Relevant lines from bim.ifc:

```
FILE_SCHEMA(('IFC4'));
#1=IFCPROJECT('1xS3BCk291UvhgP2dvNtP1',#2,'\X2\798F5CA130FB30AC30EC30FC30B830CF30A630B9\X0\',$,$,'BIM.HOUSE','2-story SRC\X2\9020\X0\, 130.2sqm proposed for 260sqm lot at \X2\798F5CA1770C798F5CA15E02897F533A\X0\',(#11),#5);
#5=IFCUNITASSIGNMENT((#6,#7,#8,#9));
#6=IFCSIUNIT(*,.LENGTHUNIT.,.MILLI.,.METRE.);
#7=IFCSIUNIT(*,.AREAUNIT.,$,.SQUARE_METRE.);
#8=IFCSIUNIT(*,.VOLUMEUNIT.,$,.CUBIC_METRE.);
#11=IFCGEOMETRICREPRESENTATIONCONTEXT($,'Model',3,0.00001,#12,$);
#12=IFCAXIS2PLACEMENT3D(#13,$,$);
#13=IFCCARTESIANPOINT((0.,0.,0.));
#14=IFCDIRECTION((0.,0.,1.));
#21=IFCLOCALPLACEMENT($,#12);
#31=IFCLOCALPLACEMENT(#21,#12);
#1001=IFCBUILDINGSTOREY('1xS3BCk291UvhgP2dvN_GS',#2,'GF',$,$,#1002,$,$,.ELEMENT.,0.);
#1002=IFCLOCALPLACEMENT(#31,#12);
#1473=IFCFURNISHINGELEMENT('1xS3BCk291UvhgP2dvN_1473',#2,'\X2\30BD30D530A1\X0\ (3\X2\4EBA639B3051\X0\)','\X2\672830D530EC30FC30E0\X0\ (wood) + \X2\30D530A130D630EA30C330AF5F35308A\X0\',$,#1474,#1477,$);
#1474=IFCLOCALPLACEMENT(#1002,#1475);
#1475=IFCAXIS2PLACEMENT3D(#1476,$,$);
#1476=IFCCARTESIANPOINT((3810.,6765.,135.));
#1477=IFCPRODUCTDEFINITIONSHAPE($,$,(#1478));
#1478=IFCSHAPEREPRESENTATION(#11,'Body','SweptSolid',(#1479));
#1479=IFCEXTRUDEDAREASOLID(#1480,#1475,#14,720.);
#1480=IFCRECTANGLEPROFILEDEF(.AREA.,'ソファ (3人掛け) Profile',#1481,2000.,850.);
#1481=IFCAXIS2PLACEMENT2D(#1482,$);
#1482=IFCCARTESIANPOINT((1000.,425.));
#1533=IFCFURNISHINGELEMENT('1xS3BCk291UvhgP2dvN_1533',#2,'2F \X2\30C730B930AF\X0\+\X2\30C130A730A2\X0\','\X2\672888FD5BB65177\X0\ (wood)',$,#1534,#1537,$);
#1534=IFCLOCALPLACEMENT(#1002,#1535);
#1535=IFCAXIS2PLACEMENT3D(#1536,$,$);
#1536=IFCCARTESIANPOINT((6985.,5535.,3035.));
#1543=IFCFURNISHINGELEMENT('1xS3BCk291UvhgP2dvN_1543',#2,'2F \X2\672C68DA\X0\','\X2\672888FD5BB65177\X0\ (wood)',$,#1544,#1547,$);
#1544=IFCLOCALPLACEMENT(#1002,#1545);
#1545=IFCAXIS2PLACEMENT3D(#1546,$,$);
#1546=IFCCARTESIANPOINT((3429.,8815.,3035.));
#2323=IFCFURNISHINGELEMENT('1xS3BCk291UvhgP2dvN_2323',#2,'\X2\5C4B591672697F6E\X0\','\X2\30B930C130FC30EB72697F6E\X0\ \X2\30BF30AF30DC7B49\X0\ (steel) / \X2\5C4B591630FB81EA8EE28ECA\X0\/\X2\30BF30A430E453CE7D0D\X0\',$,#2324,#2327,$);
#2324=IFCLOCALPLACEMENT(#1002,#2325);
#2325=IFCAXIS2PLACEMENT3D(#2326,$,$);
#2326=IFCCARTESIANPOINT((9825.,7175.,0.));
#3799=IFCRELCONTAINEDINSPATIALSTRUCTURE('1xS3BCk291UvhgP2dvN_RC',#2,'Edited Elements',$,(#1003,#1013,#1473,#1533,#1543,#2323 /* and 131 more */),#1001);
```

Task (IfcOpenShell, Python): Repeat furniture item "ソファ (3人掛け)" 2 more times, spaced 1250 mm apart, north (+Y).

```python
import numpy as np
import ifcopenshell
import ifcopenshell.api.geometry
import ifcopenshell.api.root
import ifcopenshell.util.element
import ifcopenshell.util.placement
import ifcopenshell.util.unit

model = ifcopenshell.open("bim.ifc")
unit_scale = ifcopenshell.util.unit.calculate_unit_scale(model)


def reuse_history(source, copy):
    """copy_class also copies each property set's owner history, people and application; keep the originals."""
    for rel in copy.IsDefinedBy:
        if rel.is_a("IfcRelDefinesByProperties") and (history := rel.RelatingPropertyDefinition.OwnerHistory):
            rel.RelatingPropertyDefinition.OwnerHistory = source.OwnerHistory
            ifcopenshell.util.element.remove_deep2(model, history)


source = model.by_id(1473)
base = ifcopenshell.util.placement.get_local_placement(source.ObjectPlacement)
step = np.array([0.0, 1.0, 0.0]) * 1.25 / unit_scale

for i in range(1, 3):
    copy = ifcopenshell.api.root.copy_class(model, product=source)
    copy.Representation = ifcopenshell.util.element.copy_deep(
        model, source.Representation, exclude=["IfcGeometricRepresentationContext", "IfcRepresentationMap"]
    )
    reuse_history(source, copy)
    matrix = base.copy()
    matrix[:3, 3] += i * step
    print("added at", matrix[:3, 3].round(3) + 0.0)
    ifcopenshell.api.geometry.edit_object_placement(model, product=copy, matrix=matrix, is_si=False)

model.write("bim_edited.ifc")
```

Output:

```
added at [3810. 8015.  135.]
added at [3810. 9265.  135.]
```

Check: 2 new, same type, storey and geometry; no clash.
